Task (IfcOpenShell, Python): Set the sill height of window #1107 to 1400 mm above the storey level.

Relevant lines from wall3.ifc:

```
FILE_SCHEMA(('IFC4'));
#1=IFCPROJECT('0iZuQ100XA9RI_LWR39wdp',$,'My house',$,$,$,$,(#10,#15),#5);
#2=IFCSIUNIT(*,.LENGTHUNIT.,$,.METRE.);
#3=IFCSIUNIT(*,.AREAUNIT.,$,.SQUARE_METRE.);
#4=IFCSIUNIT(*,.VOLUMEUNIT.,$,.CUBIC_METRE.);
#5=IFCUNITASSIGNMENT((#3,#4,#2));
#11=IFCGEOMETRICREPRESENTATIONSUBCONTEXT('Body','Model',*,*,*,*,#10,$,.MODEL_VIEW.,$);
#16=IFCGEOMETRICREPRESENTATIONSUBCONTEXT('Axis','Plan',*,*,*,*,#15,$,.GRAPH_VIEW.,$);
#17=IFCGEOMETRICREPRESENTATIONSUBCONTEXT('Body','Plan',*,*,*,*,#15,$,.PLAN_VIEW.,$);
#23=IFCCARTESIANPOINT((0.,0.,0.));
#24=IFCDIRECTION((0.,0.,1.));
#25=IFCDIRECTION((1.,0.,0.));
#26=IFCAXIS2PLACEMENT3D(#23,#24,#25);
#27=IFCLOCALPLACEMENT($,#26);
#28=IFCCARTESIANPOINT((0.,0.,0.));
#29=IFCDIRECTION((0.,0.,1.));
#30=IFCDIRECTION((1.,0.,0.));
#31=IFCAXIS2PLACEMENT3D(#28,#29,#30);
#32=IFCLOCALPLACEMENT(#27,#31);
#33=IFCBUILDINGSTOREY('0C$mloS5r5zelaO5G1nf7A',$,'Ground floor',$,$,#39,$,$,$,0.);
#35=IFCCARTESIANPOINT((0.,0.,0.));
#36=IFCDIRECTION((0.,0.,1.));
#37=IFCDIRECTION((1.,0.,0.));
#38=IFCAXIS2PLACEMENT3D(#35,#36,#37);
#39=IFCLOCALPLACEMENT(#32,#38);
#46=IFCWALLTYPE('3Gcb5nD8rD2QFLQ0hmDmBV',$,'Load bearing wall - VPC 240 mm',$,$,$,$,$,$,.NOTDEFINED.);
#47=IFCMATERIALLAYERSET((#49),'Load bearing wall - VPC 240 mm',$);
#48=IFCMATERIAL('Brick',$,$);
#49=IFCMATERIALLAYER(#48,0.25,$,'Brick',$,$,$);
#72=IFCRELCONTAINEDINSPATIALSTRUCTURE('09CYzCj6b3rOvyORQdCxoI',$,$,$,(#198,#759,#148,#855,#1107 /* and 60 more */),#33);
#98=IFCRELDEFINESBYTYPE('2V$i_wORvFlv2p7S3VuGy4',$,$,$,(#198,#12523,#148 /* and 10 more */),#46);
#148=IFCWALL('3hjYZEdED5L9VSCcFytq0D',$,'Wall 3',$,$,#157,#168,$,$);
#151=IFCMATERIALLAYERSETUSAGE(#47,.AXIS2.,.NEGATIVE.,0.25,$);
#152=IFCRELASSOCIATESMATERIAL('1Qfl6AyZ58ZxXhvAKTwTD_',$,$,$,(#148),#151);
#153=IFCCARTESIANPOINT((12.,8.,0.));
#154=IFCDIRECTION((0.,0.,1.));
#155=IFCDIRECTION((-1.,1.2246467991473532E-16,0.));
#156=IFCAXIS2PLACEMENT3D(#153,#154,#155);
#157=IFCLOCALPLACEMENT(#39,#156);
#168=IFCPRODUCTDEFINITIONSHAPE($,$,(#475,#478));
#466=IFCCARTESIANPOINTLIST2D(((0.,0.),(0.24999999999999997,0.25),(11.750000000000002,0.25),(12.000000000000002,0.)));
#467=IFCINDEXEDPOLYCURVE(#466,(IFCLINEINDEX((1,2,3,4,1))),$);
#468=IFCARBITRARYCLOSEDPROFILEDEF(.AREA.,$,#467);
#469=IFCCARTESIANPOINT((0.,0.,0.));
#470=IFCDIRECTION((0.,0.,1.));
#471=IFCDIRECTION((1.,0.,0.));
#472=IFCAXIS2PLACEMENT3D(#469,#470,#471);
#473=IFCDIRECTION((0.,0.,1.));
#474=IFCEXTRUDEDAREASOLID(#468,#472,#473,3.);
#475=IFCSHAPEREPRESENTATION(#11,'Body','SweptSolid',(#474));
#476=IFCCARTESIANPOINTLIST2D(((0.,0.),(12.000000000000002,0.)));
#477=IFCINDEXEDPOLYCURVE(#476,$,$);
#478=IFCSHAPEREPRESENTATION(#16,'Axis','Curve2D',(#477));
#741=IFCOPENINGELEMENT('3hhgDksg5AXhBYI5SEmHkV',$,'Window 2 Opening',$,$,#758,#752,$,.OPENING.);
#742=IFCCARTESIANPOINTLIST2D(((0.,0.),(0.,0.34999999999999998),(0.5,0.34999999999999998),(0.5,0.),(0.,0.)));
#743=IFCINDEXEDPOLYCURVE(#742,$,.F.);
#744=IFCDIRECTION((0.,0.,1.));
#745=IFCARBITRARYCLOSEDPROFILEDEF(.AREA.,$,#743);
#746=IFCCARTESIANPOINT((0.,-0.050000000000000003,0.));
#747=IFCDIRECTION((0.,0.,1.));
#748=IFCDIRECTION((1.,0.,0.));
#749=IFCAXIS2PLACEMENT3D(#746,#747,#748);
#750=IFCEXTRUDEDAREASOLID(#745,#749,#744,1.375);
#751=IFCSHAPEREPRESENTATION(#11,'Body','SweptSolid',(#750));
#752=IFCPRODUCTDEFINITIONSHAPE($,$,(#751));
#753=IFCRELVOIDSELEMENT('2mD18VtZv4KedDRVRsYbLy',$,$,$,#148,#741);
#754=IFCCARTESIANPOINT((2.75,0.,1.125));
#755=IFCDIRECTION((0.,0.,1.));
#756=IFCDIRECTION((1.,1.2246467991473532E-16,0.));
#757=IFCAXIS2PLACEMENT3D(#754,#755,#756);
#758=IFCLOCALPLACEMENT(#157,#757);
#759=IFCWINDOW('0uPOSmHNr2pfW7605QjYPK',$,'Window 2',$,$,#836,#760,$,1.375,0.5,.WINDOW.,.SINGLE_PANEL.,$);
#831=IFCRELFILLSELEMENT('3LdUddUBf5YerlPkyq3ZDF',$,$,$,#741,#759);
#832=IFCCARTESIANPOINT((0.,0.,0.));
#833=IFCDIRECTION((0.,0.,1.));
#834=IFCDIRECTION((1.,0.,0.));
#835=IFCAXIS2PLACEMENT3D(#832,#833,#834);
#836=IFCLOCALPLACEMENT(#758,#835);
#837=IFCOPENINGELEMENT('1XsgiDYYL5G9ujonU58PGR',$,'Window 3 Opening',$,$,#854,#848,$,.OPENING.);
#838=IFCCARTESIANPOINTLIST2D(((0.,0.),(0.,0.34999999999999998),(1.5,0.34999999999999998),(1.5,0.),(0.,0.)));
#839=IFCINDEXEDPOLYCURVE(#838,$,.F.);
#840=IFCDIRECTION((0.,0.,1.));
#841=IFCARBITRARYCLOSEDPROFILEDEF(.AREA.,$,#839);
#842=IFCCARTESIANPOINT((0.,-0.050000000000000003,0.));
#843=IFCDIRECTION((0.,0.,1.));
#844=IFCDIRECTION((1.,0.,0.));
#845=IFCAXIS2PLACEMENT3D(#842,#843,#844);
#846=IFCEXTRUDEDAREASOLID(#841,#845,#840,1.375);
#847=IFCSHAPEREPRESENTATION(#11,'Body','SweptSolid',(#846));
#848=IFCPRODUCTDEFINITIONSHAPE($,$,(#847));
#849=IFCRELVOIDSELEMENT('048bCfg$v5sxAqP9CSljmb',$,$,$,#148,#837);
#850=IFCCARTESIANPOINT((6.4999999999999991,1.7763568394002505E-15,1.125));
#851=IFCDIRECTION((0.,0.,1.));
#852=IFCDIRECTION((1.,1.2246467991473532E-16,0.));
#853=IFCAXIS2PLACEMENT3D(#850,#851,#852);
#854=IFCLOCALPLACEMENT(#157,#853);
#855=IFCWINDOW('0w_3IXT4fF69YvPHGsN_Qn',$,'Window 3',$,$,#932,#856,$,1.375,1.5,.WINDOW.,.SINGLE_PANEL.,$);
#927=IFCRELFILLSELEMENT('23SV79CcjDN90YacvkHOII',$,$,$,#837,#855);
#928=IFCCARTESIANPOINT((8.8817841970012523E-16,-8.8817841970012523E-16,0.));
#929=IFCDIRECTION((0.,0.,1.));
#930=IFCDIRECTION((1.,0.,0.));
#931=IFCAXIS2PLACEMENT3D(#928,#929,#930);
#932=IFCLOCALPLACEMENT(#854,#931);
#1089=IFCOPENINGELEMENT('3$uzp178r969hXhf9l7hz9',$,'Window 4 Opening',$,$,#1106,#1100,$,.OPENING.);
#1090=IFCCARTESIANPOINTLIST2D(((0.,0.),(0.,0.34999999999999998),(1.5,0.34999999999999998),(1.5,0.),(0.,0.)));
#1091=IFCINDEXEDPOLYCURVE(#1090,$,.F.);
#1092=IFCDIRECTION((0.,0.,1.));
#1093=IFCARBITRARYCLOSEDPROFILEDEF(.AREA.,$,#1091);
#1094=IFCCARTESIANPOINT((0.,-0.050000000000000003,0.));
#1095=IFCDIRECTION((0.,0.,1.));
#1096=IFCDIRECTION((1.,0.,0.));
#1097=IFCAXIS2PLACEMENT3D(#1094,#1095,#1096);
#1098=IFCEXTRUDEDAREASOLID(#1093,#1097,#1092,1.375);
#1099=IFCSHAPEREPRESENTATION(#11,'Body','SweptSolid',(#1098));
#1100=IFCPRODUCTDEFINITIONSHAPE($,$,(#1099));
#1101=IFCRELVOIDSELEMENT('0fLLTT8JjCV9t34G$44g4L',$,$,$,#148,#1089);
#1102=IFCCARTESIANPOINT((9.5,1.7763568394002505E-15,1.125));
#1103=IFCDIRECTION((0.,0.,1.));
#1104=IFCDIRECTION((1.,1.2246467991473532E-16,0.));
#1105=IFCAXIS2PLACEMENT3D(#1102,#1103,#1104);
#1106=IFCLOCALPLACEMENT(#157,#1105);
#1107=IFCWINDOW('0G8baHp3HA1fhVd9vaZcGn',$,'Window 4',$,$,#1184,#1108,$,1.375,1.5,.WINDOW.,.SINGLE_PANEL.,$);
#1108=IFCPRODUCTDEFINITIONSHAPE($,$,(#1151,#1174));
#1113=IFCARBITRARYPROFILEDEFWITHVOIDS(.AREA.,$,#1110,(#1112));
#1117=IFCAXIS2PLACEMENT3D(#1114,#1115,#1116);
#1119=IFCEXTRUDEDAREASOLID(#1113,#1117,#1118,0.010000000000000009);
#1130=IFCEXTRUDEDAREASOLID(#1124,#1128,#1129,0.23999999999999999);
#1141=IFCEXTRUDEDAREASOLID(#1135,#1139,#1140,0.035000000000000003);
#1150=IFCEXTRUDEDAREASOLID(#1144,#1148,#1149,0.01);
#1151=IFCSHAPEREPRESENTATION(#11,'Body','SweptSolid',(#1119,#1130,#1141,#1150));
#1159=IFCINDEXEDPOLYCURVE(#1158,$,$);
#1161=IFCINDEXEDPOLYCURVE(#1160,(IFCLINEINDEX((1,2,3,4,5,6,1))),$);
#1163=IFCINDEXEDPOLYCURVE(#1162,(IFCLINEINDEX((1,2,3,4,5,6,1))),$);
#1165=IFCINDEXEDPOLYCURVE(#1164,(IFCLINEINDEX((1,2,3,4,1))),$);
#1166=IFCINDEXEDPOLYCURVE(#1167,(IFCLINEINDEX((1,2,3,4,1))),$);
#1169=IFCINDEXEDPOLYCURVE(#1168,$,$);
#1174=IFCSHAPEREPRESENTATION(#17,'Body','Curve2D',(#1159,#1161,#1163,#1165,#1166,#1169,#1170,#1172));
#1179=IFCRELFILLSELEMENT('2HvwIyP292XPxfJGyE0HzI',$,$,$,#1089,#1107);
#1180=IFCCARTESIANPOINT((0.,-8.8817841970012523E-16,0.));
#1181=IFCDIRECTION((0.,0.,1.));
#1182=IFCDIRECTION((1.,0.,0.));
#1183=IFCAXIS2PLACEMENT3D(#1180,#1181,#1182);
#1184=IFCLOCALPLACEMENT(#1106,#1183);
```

```python
import numpy as np
import ifcopenshell
import ifcopenshell.api.geometry
import ifcopenshell.geom
import ifcopenshell.util.element
import ifcopenshell.util.placement
import ifcopenshell.util.shape
import ifcopenshell.util.unit

model = ifcopenshell.open("wall3.ifc")
unit_scale = ifcopenshell.util.unit.calculate_unit_scale(model)

window = model.by_guid("0G8baHp3HA1fhVd9vaZcGn")
opening = window.FillsVoids[0].RelatingOpeningElement
storey = ifcopenshell.util.element.get_container(window, ifc_class="IfcBuildingStorey")
level = ifcopenshell.util.placement.get_local_placement(storey.ObjectPlacement)[2, 3]

# The opening's origin need not be at the sill, so measure its lowest point.
shape = ifcopenshell.geom.create_shape(ifcopenshell.geom.settings(), opening)
bottom = ifcopenshell.util.shape.get_shape_bottom_elevation(shape, shape.geometry) / unit_scale
dz = level + 1.4 / unit_scale - bottom

shift = np.array([0.0, 0.0, dz])
# The window is placed relative to its opening, so it follows when the opening moves.
matrix = ifcopenshell.util.placement.get_local_placement(opening.ObjectPlacement)
matrix[:3, 3] += shift
ifcopenshell.api.geometry.edit_object_placement(
    model, product=opening, matrix=matrix, is_si=False, should_transform_children=True
)

print(f"moved by {dz * unit_scale:+.3f} m")

model.write("wall3_v2.ifc")
```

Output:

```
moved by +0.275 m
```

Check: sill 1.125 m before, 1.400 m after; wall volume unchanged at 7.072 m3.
